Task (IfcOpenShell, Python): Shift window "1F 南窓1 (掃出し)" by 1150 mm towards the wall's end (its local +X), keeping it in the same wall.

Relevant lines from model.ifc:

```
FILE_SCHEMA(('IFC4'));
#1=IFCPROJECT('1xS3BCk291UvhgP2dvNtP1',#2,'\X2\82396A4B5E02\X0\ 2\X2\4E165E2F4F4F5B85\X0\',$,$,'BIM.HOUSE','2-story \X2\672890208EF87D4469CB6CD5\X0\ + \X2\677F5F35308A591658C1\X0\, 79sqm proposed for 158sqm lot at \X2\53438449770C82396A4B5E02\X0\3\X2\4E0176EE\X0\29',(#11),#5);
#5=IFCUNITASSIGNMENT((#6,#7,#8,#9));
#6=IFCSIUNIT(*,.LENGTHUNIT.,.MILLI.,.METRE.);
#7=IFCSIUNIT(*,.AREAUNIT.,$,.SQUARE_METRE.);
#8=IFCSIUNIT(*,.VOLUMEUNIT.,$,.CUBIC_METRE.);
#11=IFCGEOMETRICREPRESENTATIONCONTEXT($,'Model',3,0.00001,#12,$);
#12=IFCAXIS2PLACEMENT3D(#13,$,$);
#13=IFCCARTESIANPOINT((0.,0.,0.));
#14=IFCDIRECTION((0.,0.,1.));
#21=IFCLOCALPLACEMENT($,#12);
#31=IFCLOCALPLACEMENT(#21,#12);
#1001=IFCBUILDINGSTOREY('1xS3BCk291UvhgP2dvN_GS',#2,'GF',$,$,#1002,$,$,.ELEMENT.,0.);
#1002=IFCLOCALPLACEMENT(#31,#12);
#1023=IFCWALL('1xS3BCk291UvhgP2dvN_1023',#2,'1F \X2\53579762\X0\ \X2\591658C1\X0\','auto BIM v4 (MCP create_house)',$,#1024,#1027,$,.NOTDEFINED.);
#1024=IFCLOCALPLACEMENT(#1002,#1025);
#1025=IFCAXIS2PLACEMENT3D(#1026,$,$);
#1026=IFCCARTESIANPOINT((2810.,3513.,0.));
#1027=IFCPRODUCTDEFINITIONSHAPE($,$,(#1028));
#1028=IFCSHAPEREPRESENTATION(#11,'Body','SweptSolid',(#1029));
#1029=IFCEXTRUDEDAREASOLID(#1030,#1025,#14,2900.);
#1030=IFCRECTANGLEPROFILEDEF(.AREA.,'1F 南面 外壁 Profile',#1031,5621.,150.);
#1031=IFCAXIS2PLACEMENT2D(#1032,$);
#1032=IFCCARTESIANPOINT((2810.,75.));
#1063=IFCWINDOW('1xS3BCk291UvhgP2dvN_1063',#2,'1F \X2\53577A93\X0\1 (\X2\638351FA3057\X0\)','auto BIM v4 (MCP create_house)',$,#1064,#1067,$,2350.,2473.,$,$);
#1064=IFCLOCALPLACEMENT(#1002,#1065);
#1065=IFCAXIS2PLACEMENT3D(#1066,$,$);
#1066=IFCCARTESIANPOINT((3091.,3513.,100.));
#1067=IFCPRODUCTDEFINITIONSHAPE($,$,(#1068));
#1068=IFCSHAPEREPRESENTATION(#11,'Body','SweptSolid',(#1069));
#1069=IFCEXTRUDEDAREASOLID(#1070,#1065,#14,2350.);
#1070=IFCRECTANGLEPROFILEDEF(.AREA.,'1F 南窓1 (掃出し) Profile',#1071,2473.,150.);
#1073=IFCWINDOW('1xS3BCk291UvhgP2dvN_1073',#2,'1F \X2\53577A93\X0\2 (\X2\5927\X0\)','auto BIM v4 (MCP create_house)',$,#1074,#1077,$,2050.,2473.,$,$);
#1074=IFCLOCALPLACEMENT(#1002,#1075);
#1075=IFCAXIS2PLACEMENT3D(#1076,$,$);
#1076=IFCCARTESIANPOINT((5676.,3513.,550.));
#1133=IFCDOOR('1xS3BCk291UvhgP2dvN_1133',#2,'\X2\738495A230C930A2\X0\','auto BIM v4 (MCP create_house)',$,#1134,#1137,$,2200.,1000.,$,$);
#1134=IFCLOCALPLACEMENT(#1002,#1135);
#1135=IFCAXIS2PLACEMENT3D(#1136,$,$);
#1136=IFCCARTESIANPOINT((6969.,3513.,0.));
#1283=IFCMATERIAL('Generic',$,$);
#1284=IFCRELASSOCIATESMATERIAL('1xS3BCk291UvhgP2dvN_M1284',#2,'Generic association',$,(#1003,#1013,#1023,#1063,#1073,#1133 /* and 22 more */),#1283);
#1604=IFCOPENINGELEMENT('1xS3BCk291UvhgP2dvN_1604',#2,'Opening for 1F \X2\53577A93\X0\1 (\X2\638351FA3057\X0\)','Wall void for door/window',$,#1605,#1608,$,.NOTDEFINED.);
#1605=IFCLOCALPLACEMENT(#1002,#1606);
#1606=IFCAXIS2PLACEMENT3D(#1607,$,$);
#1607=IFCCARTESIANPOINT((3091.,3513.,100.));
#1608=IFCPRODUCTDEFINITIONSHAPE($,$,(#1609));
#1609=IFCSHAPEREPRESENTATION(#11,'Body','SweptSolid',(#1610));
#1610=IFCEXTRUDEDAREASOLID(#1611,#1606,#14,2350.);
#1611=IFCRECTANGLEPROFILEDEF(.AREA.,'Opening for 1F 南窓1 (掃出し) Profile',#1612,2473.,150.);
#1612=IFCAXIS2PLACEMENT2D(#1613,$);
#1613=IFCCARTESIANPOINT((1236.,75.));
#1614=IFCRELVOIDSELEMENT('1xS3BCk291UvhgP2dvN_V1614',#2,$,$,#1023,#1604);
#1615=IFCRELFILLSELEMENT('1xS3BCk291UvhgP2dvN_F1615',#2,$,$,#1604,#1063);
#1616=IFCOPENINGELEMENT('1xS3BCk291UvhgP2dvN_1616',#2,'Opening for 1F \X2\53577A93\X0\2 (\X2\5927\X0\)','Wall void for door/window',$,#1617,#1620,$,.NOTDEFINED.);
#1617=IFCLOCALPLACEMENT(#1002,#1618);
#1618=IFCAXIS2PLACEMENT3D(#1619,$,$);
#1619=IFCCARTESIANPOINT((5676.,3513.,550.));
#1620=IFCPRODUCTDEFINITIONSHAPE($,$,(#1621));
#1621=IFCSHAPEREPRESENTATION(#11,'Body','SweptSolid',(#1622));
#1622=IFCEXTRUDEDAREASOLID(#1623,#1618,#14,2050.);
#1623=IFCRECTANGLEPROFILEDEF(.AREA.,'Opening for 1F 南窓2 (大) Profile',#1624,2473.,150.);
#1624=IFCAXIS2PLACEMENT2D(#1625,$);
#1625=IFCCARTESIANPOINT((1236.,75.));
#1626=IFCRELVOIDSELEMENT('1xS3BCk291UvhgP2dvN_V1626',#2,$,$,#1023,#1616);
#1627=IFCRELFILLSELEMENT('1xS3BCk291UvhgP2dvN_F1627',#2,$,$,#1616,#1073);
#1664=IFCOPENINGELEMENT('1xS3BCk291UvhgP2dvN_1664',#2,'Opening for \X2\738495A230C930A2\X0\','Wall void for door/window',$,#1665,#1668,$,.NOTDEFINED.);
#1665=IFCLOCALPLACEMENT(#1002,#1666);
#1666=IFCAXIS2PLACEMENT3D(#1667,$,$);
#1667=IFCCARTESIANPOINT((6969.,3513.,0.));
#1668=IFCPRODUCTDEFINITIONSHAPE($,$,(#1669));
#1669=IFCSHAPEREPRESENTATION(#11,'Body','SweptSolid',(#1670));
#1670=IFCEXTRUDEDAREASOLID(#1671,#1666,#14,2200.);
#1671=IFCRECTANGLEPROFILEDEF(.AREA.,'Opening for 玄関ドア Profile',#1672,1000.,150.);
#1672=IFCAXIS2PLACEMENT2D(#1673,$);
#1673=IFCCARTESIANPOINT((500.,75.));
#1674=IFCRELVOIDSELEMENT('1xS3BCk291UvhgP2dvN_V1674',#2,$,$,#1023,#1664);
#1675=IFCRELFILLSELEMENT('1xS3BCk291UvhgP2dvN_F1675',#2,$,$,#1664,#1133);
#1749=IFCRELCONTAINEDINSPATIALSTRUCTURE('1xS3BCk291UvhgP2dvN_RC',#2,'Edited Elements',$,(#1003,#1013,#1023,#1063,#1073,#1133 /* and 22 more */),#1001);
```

```python
import ifcopenshell
import ifcopenshell.api.geometry
import ifcopenshell.util.placement
import ifcopenshell.util.unit

model = ifcopenshell.open("model.ifc")
unit_scale = ifcopenshell.util.unit.calculate_unit_scale(model)

window = model.by_guid("1xS3BCk291UvhgP2dvN_1063")
opening = window.FillsVoids[0].RelatingOpeningElement
wall = opening.VoidsElements[0].RelatingBuildingElement

wall_matrix = ifcopenshell.util.placement.get_local_placement(wall.ObjectPlacement)
shift = wall_matrix[:3, 0] * 1.15 / unit_scale
before = ifcopenshell.util.placement.get_local_placement(window.ObjectPlacement)[:3, 3].copy()

# The window is not placed relative to its opening, so move both.
for product in (opening, window):
    matrix = ifcopenshell.util.placement.get_local_placement(product.ObjectPlacement)
    matrix[:3, 3] += shift
    ifcopenshell.api.geometry.edit_object_placement(model, product=product, matrix=matrix, is_si=False)

after = ifcopenshell.util.placement.get_local_placement(window.ObjectPlacement)[:3, 3]
print("window moved by", (after - before).round(3) + 0.0)

model.write("model-out.ifc")
```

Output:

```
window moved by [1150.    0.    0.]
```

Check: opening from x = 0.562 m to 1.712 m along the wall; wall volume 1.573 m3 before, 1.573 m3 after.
